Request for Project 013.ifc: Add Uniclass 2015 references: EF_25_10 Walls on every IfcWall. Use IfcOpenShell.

First a look at what the model holds.

```python
import ifcopenshell

model = ifcopenshell.open("Project 013.ifc")
print(model.schema)
print("classifications:", [c.Name for c in model.by_type("IfcClassification")])
for ifc_class in ("IfcDoor", "IfcRoof", "IfcStair", "IfcWall", "IfcWindow"):
    print(ifc_class, len(model.by_type(ifc_class)))
```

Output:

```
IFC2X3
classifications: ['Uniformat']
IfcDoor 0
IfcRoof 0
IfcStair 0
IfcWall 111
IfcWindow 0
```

```python
import ifcopenshell
import ifcopenshell.api.classification

model = ifcopenshell.open("Project 013.ifc")

# IFC2X3 requires Source and Edition and has no link from the project to the system.
system = model.create_entity("IfcClassification", Source="NBS", Edition="2015", Name="Uniclass 2015")

codes = {
    "IfcWall": ("EF_25_10", "Walls"),
}
for ifc_class, (code, name) in codes.items():
    products = model.by_type(ifc_class)
    ifcopenshell.api.classification.add_reference(
        model, products=products, classification=system, identification=code, name=name
    )
    print(code, len(products))

model.write("Project 013_v2.ifc")
```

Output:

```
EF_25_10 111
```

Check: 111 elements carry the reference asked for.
